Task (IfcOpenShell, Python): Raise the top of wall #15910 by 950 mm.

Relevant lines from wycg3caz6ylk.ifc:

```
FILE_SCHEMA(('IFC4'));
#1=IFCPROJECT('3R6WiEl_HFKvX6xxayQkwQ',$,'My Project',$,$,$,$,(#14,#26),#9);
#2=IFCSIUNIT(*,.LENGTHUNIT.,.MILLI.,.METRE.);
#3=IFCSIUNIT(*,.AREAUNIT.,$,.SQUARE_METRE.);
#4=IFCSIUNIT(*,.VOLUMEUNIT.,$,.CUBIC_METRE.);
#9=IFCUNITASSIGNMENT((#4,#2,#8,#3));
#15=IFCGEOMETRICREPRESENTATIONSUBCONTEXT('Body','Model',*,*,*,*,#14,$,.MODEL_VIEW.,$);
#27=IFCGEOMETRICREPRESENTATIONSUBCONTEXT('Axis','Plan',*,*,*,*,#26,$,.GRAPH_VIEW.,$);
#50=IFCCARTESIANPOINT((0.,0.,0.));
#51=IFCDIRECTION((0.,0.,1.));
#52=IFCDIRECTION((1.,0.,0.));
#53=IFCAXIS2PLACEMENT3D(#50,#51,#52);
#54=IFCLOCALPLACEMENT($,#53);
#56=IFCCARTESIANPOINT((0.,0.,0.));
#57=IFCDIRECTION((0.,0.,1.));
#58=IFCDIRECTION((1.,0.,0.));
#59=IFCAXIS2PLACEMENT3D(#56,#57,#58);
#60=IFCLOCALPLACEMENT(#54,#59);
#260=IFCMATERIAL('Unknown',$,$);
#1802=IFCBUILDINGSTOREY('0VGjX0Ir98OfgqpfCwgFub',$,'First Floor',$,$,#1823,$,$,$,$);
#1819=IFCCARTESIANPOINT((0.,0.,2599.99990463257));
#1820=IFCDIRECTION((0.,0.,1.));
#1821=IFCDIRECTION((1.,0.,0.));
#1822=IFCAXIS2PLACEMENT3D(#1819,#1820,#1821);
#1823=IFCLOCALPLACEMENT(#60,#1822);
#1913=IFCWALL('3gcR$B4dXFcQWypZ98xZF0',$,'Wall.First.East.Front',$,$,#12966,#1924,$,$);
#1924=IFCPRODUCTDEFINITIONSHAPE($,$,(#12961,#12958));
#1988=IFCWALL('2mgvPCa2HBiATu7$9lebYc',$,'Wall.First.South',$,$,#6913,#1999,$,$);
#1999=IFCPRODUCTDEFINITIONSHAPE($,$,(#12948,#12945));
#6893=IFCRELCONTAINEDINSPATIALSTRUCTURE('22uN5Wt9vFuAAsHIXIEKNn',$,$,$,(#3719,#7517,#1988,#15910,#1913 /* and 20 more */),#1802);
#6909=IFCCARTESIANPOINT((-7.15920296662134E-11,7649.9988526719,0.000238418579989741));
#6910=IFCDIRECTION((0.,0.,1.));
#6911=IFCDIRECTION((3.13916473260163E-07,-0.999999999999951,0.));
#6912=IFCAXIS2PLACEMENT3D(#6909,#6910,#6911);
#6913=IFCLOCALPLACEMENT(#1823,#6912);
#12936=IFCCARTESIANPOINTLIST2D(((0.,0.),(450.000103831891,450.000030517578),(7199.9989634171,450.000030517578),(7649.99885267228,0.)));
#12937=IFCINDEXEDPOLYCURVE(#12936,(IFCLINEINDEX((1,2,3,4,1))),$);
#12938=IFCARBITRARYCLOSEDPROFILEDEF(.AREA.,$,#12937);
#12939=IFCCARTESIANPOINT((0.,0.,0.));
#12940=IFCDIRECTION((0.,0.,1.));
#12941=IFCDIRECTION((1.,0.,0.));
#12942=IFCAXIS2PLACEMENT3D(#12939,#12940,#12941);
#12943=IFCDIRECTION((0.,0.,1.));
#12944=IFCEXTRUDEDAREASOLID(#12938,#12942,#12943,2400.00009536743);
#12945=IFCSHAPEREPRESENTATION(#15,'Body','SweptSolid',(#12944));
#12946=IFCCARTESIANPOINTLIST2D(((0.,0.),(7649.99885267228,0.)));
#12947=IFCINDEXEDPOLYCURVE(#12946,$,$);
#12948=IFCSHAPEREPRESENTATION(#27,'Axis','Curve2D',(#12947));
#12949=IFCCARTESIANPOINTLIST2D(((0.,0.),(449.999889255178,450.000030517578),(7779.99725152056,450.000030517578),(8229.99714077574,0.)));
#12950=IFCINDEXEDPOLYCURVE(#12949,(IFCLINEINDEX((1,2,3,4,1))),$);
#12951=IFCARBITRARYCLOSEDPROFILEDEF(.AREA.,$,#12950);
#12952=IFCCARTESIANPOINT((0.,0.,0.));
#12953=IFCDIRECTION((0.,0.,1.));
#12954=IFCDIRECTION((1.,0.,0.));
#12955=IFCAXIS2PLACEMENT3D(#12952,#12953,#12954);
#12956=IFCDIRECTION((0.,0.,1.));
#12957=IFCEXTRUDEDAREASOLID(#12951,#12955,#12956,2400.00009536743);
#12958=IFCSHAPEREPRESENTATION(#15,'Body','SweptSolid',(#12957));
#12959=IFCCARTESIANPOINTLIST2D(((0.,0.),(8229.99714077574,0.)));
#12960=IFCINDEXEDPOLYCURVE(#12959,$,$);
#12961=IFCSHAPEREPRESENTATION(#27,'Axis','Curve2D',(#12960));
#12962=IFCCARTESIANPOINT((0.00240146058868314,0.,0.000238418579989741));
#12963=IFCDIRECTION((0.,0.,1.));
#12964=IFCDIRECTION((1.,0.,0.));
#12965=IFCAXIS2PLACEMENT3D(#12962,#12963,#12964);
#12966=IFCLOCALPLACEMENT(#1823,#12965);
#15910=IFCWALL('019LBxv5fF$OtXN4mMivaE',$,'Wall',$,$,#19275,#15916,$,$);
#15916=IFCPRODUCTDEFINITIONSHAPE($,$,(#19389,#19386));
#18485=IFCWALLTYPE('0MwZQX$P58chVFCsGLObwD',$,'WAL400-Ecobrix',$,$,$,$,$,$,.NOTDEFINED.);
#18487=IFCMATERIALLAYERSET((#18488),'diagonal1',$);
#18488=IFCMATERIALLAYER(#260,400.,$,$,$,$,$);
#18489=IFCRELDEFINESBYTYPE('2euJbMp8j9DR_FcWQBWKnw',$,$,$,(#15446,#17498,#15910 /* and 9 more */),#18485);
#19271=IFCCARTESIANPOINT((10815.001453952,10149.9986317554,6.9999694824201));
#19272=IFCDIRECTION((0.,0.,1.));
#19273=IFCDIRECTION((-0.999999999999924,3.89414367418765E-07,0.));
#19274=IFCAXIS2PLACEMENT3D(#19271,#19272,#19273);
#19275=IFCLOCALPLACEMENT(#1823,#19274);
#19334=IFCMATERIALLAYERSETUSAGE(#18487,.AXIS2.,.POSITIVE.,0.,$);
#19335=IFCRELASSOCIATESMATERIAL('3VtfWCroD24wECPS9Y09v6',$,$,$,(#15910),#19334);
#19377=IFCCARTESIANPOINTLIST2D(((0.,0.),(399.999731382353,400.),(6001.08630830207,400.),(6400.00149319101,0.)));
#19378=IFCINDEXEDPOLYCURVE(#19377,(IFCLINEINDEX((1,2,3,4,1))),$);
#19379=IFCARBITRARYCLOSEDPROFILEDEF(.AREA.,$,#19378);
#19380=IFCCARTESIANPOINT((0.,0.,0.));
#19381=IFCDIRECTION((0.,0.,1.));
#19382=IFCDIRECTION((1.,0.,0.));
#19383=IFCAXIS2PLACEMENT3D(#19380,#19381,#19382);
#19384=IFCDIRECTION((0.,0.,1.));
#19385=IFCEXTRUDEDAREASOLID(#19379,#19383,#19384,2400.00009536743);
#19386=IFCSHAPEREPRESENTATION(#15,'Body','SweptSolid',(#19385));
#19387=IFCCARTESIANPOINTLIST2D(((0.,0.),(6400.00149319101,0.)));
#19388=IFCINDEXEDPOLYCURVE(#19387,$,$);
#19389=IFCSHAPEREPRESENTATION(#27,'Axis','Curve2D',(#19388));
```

```python
import ifcopenshell
import ifcopenshell.geom
import ifcopenshell.util.representation
import ifcopenshell.util.shape
import ifcopenshell.util.unit

model = ifcopenshell.open("wycg3caz6ylk.ifc")
unit_scale = ifcopenshell.util.unit.calculate_unit_scale(model)
settings = ifcopenshell.geom.settings()


def volume(element):
    """Net volume in cubic metres, openings subtracted."""
    shape = ifcopenshell.geom.create_shape(settings, element)
    return ifcopenshell.util.shape.get_volume(shape.geometry)


wall = model.by_guid("019LBxv5fF$OtXN4mMivaE")
before = volume(wall)

body = ifcopenshell.util.representation.get_representation(wall, "Model", "Body")
solid = body.Items[0]
old_height = solid.Depth
solid.Depth += 0.95 / unit_scale
after = volume(wall)

print(f"height {old_height:g} -> {solid.Depth:g}, volume {before:.3f} -> {after:.3f} m3")

model.write("wycg3caz6ylk_rev.ifc")
```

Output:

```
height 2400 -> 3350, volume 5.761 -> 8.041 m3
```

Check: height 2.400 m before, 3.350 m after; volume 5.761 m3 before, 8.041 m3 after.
